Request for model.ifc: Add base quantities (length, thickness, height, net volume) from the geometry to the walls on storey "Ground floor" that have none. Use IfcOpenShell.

First a look at what the model holds.

```python
import ifcopenshell
import ifcopenshell.util.element
import ifcopenshell.util.unit

model = ifcopenshell.open("model.ifc")
print(model.schema)
for unit_type in ("LENGTHUNIT", "AREAUNIT", "VOLUMEUNIT"):
    print(unit_type, ifcopenshell.util.unit.calculate_unit_scale(model, unit_type))
storey = next(s for s in model.by_type("IfcBuildingStorey") if s.Name == "Ground floor")
walls = [e for e in ifcopenshell.util.element.get_decomposition(storey) if e.is_a("IfcWall")]
for e in sorted(walls, key=lambda e: e.id()):
    print(e.id(), e.is_a(), e.Name, list(ifcopenshell.util.element.get_psets(e, qtos_only=True)), sep=" | ")
```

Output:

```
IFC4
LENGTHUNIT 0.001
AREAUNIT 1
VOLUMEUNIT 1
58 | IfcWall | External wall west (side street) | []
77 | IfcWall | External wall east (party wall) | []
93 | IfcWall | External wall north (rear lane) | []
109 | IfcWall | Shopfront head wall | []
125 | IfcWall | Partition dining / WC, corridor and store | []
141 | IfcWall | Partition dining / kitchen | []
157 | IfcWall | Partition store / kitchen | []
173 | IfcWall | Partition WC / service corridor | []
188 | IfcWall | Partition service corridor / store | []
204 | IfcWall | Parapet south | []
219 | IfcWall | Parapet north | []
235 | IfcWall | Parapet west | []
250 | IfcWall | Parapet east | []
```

```python
import ifcopenshell
import ifcopenshell.api.pset
import ifcopenshell.geom
import ifcopenshell.util.element
import ifcopenshell.util.shape
import ifcopenshell.util.unit

model = ifcopenshell.open("model.ifc")
unit_scale = ifcopenshell.util.unit.calculate_unit_scale(model)
volume_scale = ifcopenshell.util.unit.calculate_unit_scale(model, "VOLUMEUNIT")
settings = ifcopenshell.geom.settings()

storey = next(s for s in model.by_type("IfcBuildingStorey") if s.Name == "Ground floor")
walls = [e for e in ifcopenshell.util.element.get_decomposition(storey) if e.is_a("IfcWall")]

for e in sorted(walls, key=lambda e: e.id()):
    if ifcopenshell.util.element.get_psets(e, qtos_only=True, should_inherit=False):
        continue
    # Geometry comes back in metres, in the element's own axes.
    shape = ifcopenshell.geom.create_shape(settings, e)
    values = {
        "Length": ifcopenshell.util.shape.get_x(shape.geometry) / unit_scale,
        "Width": ifcopenshell.util.shape.get_y(shape.geometry) / unit_scale,
        "Height": ifcopenshell.util.shape.get_z(shape.geometry) / unit_scale,
        "NetVolume": ifcopenshell.util.shape.get_volume(shape.geometry) / volume_scale,
    }
    qto = ifcopenshell.api.pset.add_qto(model, product=e, name="Qto_WallBaseQuantities")
    ifcopenshell.api.pset.edit_qto(model, qto=qto, properties=values)
    print(e.id(), {k: round(v, 3) for k, v in values.items()})

model.write("model-out.ifc")
```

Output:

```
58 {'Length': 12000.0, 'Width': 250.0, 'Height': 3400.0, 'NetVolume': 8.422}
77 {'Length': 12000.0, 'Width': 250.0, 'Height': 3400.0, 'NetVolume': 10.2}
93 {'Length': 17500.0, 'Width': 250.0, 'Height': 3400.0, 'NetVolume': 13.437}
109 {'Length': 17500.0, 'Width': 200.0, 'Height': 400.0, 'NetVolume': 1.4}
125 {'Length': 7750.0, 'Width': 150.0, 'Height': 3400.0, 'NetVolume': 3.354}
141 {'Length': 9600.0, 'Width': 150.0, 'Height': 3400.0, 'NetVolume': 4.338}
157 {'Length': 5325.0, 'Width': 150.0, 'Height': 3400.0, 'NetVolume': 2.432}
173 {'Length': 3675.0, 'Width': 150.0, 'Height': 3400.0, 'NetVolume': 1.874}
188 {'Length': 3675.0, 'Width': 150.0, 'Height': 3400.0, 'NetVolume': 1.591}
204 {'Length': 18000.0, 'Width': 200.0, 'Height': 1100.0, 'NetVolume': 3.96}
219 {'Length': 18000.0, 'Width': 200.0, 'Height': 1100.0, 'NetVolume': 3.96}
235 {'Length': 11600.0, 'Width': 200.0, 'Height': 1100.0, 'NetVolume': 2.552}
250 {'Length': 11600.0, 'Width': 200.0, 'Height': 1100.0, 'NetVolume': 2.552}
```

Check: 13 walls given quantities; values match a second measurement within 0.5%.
